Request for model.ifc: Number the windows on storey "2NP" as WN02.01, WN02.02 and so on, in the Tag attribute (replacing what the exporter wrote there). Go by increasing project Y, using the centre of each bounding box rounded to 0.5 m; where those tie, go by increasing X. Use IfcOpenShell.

First a look at what the model holds.

```python
import ifcopenshell
import ifcopenshell.util.element
import ifcopenshell.util.placement

model = ifcopenshell.open("model.ifc")
print(model.schema)
storey = next(s for s in model.by_type("IfcBuildingStorey") if s.Name == "2NP")
windows = [e for e in ifcopenshell.util.element.get_decomposition(storey) if e.is_a("IfcWindow")]
for e in sorted(windows, key=lambda e: e.id()):
    origin = ifcopenshell.util.placement.get_local_placement(e.ObjectPlacement)[:3, 3]
    print(e.id(), e.Tag, e.Name, origin.round(2) + 0.0, sep=" | ")
```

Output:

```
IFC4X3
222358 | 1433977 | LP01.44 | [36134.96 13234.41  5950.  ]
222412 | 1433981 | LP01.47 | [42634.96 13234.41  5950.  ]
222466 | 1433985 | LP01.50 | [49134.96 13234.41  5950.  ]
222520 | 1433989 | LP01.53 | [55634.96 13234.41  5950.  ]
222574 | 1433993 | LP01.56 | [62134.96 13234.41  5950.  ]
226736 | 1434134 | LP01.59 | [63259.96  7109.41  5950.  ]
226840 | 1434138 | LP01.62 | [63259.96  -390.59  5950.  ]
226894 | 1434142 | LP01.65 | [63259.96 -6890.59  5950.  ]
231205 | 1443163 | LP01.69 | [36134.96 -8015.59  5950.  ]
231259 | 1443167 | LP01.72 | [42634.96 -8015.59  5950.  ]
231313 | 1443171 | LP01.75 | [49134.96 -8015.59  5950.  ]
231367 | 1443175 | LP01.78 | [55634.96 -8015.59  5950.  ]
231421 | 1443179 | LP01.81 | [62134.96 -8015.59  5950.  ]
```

```python
import ifcopenshell
import ifcopenshell.geom
import ifcopenshell.util.element
import ifcopenshell.util.shape

model = ifcopenshell.open("model.ifc")
settings = ifcopenshell.geom.settings()
settings.set("use-world-coords", True)


def centre(element):
    shape = ifcopenshell.geom.create_shape(settings, element)
    return ifcopenshell.util.shape.get_bbox_centroid(shape.geometry)


storey = next(s for s in model.by_type("IfcBuildingStorey") if s.Name == "2NP")
windows = [e for e in ifcopenshell.util.element.get_decomposition(storey) if e.is_a("IfcWindow")]

# Insertion points can sit at a corner or the storey origin, so sort by the geometry (in metres).
centres = {e: centre(e) for e in windows}
windows.sort(key=lambda e: (round(centres[e][1] / 0.5), centres[e][0]))

for i, e in enumerate(windows, start=1):
    number = f"WN02.{i:02d}"
    e.Tag = number
    print(e.id(), number)

model.write("model_updated.ifc")
```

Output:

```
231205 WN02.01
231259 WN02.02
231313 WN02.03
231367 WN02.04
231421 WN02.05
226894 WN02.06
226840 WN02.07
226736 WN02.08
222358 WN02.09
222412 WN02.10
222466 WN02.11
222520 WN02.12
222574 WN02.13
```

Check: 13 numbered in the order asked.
